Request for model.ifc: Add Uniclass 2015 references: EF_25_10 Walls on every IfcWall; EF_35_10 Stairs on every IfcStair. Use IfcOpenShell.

First a look at what the model holds.

```python
import ifcopenshell

model = ifcopenshell.open("model.ifc")
print(model.schema)
print("classifications:", [c.Name for c in model.by_type("IfcClassification")])
for ifc_class in ("IfcDoor", "IfcRoof", "IfcStair", "IfcWall", "IfcWindow"):
    print(ifc_class, len(model.by_type(ifc_class)))
```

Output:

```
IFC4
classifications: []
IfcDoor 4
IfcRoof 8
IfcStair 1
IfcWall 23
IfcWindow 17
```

```python
import ifcopenshell
import ifcopenshell.api.classification

model = ifcopenshell.open("model.ifc")

system = ifcopenshell.api.classification.add_classification(model, classification="Uniclass 2015")

codes = {
    "IfcWall": ("EF_25_10", "Walls"),
    "IfcStair": ("EF_35_10", "Stairs"),
}
for ifc_class, (code, name) in codes.items():
    products = model.by_type(ifc_class)
    ifcopenshell.api.classification.add_reference(
        model, products=products, classification=system, identification=code, name=name
    )
    print(code, len(products))

model.write("model_updated.ifc")
```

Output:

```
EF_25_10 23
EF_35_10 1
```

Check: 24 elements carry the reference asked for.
